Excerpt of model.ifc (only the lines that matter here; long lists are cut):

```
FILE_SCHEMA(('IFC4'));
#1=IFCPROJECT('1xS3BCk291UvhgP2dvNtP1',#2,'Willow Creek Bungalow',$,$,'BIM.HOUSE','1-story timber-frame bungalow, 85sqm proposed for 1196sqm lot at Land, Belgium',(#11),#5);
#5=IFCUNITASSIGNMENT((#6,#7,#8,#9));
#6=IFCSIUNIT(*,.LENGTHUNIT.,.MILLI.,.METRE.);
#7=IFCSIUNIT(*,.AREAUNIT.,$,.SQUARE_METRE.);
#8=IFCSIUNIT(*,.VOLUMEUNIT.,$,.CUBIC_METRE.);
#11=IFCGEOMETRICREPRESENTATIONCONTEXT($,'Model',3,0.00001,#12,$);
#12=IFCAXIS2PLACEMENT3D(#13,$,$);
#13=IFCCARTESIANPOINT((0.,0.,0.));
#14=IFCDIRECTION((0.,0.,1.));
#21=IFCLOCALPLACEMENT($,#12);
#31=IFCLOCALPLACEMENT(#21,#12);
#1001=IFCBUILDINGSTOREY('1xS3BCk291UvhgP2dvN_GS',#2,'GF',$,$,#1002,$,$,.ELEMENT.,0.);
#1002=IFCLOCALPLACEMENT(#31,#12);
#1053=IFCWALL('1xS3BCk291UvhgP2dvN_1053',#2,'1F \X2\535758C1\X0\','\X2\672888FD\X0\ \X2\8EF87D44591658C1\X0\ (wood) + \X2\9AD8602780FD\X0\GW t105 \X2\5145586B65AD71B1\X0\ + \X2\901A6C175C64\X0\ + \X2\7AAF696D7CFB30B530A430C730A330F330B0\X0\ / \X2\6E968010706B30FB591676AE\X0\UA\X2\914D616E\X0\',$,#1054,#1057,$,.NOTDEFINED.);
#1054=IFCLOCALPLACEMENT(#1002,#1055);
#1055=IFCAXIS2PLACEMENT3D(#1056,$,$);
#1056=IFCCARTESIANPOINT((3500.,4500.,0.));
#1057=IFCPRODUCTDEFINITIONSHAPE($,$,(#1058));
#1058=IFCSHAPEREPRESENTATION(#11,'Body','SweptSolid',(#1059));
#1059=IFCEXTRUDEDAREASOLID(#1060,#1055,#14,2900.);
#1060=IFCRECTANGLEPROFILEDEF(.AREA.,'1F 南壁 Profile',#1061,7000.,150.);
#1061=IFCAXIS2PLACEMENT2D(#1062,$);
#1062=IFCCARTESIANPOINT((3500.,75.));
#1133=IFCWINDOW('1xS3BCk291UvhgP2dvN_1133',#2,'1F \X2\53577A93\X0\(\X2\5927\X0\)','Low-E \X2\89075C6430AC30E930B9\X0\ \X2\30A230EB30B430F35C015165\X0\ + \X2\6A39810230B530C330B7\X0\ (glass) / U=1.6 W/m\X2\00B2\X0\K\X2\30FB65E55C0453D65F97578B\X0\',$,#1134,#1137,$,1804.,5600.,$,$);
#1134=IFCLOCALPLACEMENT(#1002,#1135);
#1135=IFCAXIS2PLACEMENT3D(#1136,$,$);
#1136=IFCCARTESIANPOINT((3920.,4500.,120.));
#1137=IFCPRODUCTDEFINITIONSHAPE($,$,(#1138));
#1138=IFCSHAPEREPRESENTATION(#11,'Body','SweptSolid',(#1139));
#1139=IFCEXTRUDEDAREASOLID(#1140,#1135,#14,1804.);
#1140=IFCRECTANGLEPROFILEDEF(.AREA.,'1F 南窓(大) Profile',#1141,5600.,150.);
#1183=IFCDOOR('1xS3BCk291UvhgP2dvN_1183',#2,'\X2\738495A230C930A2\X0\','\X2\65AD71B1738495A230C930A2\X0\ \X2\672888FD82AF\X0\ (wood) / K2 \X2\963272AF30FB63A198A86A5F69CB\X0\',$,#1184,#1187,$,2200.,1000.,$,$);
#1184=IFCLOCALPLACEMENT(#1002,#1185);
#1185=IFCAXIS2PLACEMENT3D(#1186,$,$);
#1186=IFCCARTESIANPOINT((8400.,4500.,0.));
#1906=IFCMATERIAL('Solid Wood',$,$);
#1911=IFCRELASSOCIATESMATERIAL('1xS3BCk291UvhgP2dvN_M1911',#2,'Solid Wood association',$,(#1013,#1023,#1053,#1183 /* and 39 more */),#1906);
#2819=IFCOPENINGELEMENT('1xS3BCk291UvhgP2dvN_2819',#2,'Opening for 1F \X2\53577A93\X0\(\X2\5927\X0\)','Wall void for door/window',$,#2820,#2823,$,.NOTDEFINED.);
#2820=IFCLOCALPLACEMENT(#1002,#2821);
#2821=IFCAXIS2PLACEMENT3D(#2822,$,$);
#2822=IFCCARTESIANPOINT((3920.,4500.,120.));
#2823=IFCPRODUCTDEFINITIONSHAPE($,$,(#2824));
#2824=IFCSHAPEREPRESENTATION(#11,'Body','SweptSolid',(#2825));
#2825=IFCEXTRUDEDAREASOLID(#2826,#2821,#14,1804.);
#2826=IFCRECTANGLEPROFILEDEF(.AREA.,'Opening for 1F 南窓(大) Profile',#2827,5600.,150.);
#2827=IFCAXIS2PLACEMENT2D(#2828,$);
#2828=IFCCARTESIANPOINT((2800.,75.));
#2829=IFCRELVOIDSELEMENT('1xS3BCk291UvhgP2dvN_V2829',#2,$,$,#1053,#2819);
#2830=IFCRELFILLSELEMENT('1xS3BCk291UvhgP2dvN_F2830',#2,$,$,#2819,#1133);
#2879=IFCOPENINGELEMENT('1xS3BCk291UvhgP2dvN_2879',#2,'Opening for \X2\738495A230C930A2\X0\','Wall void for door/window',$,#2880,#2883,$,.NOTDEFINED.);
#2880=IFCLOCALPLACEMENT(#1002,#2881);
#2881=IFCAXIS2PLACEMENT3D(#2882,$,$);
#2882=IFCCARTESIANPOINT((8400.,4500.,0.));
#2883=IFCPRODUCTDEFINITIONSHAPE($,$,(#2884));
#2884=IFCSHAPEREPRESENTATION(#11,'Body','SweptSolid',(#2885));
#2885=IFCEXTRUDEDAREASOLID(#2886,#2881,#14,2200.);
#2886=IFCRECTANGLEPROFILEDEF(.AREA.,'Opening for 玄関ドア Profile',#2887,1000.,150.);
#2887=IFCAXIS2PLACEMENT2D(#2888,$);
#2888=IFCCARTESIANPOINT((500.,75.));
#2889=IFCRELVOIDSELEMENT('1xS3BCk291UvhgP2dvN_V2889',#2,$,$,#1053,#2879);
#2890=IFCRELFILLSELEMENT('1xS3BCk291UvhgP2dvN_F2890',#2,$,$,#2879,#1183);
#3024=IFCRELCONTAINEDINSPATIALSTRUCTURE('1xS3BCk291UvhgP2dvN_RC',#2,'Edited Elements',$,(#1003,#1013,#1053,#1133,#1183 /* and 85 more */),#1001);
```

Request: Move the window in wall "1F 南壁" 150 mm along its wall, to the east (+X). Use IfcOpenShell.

```python
import ifcopenshell
import ifcopenshell.api.geometry
import ifcopenshell.util.placement

model = ifcopenshell.open("model.ifc")

window = model.by_guid("1xS3BCk291UvhgP2dvN_1133")
opening = window.FillsVoids[0].RelatingOpeningElement
wall = opening.VoidsElements[0].RelatingBuildingElement

wall_matrix = ifcopenshell.util.placement.get_local_placement(wall.ObjectPlacement)
shift = wall_matrix[:3, 0] * 150.0
before = ifcopenshell.util.placement.get_local_placement(window.ObjectPlacement)[:3, 3].copy()

# The window is not placed relative to its opening, so move both.
for product in (opening, window):
    matrix = ifcopenshell.util.placement.get_local_placement(product.ObjectPlacement)
    matrix[:3, 3] += shift
    ifcopenshell.api.geometry.edit_object_placement(model, product=product, matrix=matrix, is_si=False)

after = ifcopenshell.util.placement.get_local_placement(window.ObjectPlacement)[:3, 3]
print("window moved by", (after - before).round(3) + 0.0)

model.write("model_updated.ifc")
```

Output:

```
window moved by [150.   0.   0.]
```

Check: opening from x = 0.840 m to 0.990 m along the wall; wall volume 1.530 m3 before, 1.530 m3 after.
